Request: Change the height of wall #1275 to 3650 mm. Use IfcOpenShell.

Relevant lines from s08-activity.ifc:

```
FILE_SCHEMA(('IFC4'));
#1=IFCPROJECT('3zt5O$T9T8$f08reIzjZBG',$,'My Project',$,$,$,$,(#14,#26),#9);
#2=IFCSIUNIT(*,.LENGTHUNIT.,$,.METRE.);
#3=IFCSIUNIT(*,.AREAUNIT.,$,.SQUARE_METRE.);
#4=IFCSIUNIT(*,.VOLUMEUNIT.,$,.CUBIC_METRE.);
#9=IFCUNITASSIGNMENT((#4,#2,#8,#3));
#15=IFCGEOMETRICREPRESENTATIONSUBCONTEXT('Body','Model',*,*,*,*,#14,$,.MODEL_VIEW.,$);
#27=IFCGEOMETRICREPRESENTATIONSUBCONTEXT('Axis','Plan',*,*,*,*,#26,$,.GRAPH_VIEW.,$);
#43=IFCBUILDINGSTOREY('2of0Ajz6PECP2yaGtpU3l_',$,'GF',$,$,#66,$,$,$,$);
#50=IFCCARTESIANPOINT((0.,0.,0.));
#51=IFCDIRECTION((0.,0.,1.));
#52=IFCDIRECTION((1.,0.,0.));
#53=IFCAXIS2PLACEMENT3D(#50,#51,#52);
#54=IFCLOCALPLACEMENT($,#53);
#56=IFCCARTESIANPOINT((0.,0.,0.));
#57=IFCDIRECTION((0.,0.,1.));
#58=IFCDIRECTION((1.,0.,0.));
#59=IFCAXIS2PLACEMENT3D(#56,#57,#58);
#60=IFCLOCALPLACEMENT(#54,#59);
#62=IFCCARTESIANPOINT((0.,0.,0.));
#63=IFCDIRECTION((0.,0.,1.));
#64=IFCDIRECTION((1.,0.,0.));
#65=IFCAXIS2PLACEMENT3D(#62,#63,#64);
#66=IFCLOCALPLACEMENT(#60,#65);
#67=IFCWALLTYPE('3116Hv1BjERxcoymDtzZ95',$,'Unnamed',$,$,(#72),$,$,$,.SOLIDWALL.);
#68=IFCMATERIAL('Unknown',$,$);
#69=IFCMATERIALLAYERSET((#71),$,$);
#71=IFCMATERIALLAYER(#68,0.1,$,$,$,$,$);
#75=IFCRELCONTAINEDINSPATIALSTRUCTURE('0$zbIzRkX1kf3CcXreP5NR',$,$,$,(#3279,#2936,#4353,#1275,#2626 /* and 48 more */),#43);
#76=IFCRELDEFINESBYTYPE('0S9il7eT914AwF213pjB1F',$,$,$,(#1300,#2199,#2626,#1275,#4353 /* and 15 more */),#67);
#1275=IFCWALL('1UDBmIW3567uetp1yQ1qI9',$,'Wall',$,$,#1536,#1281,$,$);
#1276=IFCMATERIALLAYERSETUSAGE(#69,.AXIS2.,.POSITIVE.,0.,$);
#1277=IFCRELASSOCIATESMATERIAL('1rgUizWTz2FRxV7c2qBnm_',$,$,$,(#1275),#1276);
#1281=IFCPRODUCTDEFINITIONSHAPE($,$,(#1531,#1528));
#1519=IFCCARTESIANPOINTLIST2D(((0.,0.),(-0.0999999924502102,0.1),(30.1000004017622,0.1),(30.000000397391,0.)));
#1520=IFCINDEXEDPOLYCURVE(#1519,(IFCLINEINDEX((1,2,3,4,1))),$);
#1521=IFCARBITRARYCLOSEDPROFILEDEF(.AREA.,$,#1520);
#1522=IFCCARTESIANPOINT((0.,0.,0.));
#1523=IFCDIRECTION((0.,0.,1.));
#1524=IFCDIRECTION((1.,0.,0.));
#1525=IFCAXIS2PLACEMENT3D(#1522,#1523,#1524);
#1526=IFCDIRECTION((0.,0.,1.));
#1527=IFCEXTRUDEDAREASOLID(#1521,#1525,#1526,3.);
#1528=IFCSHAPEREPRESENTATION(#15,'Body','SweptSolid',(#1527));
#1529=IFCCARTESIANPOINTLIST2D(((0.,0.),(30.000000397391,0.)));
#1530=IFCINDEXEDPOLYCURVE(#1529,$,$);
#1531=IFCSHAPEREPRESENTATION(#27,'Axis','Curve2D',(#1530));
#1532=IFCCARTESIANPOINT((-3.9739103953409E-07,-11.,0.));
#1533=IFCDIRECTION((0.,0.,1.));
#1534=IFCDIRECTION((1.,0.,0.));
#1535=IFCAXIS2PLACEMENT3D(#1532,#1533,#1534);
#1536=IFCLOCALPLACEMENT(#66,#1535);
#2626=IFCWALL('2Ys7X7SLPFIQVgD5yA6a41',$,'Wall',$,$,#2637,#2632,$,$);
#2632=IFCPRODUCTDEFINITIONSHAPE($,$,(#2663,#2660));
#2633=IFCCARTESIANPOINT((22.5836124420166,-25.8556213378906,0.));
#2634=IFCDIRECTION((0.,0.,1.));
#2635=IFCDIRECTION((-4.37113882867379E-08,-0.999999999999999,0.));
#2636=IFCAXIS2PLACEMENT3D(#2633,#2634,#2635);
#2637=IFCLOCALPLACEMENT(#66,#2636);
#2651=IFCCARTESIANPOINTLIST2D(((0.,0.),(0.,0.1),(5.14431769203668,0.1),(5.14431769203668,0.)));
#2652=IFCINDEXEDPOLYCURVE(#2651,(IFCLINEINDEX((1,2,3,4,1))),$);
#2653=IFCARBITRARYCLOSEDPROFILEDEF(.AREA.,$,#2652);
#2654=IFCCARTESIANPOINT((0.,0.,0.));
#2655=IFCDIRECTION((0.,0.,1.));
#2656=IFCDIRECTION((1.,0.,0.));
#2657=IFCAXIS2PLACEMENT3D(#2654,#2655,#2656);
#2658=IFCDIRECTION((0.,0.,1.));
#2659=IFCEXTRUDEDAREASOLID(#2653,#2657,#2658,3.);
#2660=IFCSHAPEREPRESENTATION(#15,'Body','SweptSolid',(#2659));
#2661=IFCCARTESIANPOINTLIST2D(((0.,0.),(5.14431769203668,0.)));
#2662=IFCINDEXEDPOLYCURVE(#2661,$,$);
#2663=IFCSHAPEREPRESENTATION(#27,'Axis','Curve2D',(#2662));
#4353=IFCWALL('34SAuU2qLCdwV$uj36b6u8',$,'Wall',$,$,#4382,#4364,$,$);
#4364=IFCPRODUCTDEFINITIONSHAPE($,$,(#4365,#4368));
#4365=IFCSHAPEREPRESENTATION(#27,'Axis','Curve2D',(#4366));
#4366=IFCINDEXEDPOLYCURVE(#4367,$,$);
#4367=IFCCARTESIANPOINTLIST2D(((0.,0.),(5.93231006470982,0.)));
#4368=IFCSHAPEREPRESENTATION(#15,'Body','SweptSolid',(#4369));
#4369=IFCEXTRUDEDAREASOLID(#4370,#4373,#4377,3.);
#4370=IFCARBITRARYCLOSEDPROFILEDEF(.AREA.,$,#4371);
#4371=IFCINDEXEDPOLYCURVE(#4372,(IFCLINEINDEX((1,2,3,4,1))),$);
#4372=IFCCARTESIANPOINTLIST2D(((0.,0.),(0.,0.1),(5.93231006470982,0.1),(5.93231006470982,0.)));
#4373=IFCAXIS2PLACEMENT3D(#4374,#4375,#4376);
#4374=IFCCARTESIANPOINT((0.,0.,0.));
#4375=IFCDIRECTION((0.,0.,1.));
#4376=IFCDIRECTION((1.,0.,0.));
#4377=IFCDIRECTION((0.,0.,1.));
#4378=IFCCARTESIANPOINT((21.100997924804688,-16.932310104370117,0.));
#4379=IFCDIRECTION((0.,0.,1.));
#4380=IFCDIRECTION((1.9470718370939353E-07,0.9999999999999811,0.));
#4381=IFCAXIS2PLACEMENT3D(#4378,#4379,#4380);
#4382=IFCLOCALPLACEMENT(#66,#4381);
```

```python
import ifcopenshell
import ifcopenshell.geom
import ifcopenshell.util.representation
import ifcopenshell.util.shape
import ifcopenshell.util.unit

model = ifcopenshell.open("s08-activity.ifc")
unit_scale = ifcopenshell.util.unit.calculate_unit_scale(model)
settings = ifcopenshell.geom.settings()


def volume(element):
    """Net volume in cubic metres, openings subtracted."""
    shape = ifcopenshell.geom.create_shape(settings, element)
    return ifcopenshell.util.shape.get_volume(shape.geometry)


wall = model.by_id(1275)
before = volume(wall)

body = ifcopenshell.util.representation.get_representation(wall, "Model", "Body")
solid = body.Items[0]
old_height = solid.Depth
solid.Depth = 3.65 / unit_scale
after = volume(wall)

print(f"height {old_height:g} -> {solid.Depth:g}, volume {before:.3f} -> {after:.3f} m3")

model.write("s08-activity_v2.ifc")
```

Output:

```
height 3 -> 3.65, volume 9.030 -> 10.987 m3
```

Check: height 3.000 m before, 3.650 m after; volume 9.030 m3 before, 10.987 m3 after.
